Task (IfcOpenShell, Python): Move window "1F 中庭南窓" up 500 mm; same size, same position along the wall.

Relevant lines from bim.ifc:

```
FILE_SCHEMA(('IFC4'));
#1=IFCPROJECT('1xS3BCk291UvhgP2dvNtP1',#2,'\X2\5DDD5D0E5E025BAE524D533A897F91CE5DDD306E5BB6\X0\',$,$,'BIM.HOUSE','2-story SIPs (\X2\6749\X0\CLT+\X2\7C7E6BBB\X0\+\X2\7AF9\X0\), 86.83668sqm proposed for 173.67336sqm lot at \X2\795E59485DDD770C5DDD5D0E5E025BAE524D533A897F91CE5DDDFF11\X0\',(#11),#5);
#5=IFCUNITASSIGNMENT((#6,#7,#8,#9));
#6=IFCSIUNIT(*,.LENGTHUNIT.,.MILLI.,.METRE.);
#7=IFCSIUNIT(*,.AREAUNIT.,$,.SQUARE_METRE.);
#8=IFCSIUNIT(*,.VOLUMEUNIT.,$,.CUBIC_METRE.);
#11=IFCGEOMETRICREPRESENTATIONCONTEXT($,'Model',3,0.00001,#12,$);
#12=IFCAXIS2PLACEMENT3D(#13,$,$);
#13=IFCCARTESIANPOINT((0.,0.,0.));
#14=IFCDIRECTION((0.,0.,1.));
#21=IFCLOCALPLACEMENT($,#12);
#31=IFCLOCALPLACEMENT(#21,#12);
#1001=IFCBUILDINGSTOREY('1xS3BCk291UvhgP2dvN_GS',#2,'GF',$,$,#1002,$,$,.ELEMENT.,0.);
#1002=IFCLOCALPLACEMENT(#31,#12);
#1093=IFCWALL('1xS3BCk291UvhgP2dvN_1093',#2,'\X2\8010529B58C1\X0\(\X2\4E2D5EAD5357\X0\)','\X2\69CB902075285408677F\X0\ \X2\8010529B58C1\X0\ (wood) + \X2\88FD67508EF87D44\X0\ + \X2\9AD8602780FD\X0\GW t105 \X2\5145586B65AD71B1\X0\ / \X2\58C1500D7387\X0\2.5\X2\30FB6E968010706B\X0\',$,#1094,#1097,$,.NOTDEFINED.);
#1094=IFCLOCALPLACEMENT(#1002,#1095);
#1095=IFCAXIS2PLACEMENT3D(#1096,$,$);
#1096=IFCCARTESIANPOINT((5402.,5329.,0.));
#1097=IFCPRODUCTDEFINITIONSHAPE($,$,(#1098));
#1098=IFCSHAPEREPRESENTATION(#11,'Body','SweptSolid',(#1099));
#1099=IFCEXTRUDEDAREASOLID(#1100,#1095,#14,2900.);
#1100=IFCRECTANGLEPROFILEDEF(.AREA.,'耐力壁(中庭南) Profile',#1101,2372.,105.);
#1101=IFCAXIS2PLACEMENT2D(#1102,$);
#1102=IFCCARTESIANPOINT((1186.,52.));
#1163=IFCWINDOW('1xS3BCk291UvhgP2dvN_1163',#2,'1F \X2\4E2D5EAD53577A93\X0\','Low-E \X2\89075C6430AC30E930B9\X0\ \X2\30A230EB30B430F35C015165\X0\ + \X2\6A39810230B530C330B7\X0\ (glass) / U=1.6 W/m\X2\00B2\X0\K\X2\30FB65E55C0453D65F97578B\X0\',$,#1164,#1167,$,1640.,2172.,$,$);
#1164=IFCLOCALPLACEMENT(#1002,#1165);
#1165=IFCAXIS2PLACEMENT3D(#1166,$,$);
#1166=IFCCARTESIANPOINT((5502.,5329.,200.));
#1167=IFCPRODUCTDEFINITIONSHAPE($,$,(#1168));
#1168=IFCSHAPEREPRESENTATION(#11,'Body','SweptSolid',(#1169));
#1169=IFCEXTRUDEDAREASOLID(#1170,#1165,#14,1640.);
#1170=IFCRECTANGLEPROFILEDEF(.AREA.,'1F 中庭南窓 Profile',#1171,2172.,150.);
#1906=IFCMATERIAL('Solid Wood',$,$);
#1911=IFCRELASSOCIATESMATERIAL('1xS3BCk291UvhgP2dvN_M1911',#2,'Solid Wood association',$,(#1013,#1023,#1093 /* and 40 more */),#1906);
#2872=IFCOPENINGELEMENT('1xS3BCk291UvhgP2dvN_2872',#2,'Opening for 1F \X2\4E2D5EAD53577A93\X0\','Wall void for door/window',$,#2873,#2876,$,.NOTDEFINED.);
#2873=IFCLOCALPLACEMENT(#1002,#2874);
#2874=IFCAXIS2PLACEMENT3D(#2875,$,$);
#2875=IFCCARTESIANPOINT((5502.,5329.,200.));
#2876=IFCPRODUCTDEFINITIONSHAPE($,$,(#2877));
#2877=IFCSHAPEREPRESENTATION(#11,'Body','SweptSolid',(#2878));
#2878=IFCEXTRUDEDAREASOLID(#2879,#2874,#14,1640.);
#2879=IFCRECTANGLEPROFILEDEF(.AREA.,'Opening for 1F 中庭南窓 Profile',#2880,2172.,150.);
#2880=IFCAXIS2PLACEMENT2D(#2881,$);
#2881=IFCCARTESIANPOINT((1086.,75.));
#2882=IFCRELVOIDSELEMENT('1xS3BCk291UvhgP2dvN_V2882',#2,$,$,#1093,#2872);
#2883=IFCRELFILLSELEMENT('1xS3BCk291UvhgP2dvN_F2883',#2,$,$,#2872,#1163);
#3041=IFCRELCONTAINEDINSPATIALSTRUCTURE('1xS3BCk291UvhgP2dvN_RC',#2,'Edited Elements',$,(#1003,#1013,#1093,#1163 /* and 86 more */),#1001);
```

```python
import numpy as np
import ifcopenshell
import ifcopenshell.api.geometry
import ifcopenshell.util.placement
import ifcopenshell.util.unit

model = ifcopenshell.open("bim.ifc")
unit_scale = ifcopenshell.util.unit.calculate_unit_scale(model)

window = model.by_guid("1xS3BCk291UvhgP2dvN_1163")
opening = window.FillsVoids[0].RelatingOpeningElement
dz = 500.0

shift = np.array([0.0, 0.0, dz])
# The window is not placed relative to its opening, so move both.
for product in (opening, window):
    matrix = ifcopenshell.util.placement.get_local_placement(product.ObjectPlacement)
    matrix[:3, 3] += shift
    ifcopenshell.api.geometry.edit_object_placement(model, product=product, matrix=matrix, is_si=False)

print(f"moved by {dz * unit_scale:+.3f} m")

model.write("bim-out.ifc")
```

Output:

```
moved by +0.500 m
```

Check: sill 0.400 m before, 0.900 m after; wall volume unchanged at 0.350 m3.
